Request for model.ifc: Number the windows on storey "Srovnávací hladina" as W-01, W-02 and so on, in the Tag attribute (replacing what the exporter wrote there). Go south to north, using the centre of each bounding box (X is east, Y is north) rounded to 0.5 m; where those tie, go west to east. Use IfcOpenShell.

First a look at what the model holds.

```python
import ifcopenshell
import ifcopenshell.util.element
import ifcopenshell.util.placement

model = ifcopenshell.open("model.ifc")
print(model.schema)
storey = next(s for s in model.by_type("IfcBuildingStorey") if s.Name == "Srovnávací hladina")
windows = [e for e in ifcopenshell.util.element.get_decomposition(storey) if e.is_a("IfcWindow")]
for e in sorted(windows, key=lambda e: e.id()):
    origin = ifcopenshell.util.placement.get_local_placement(e.ObjectPlacement)[:3, 3]
    print(e.id(), e.Tag, e.Name, origin.round(2) + 0.0, sep=" | ")
```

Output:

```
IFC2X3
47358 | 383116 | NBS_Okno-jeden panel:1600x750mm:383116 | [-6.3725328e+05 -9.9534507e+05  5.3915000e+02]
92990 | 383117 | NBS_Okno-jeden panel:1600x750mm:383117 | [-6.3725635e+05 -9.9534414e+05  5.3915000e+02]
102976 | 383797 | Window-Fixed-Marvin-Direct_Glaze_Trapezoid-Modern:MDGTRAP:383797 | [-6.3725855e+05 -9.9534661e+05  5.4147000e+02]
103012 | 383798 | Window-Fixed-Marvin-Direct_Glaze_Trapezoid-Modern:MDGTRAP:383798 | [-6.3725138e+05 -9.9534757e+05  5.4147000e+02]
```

```python
import ifcopenshell
import ifcopenshell.geom
import ifcopenshell.util.element
import ifcopenshell.util.shape

model = ifcopenshell.open("model.ifc")
settings = ifcopenshell.geom.settings()
settings.set("use-world-coords", True)


def centre(element):
    shape = ifcopenshell.geom.create_shape(settings, element)
    return ifcopenshell.util.shape.get_bbox_centroid(shape.geometry)


storey = next(s for s in model.by_type("IfcBuildingStorey") if s.Name == "Srovnávací hladina")
windows = [e for e in ifcopenshell.util.element.get_decomposition(storey) if e.is_a("IfcWindow")]

# Insertion points can sit at a corner or the storey origin, so sort by the geometry (in metres).
centres = {e: centre(e) for e in windows}
windows.sort(key=lambda e: (round(centres[e][1] / 0.5), centres[e][0]))

for i, e in enumerate(windows, start=1):
    number = f"W-{i:02d}"
    e.Tag = number
    print(e.id(), number)

model.write("model_edited.ifc")
```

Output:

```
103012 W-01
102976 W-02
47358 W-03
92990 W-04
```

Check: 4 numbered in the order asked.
